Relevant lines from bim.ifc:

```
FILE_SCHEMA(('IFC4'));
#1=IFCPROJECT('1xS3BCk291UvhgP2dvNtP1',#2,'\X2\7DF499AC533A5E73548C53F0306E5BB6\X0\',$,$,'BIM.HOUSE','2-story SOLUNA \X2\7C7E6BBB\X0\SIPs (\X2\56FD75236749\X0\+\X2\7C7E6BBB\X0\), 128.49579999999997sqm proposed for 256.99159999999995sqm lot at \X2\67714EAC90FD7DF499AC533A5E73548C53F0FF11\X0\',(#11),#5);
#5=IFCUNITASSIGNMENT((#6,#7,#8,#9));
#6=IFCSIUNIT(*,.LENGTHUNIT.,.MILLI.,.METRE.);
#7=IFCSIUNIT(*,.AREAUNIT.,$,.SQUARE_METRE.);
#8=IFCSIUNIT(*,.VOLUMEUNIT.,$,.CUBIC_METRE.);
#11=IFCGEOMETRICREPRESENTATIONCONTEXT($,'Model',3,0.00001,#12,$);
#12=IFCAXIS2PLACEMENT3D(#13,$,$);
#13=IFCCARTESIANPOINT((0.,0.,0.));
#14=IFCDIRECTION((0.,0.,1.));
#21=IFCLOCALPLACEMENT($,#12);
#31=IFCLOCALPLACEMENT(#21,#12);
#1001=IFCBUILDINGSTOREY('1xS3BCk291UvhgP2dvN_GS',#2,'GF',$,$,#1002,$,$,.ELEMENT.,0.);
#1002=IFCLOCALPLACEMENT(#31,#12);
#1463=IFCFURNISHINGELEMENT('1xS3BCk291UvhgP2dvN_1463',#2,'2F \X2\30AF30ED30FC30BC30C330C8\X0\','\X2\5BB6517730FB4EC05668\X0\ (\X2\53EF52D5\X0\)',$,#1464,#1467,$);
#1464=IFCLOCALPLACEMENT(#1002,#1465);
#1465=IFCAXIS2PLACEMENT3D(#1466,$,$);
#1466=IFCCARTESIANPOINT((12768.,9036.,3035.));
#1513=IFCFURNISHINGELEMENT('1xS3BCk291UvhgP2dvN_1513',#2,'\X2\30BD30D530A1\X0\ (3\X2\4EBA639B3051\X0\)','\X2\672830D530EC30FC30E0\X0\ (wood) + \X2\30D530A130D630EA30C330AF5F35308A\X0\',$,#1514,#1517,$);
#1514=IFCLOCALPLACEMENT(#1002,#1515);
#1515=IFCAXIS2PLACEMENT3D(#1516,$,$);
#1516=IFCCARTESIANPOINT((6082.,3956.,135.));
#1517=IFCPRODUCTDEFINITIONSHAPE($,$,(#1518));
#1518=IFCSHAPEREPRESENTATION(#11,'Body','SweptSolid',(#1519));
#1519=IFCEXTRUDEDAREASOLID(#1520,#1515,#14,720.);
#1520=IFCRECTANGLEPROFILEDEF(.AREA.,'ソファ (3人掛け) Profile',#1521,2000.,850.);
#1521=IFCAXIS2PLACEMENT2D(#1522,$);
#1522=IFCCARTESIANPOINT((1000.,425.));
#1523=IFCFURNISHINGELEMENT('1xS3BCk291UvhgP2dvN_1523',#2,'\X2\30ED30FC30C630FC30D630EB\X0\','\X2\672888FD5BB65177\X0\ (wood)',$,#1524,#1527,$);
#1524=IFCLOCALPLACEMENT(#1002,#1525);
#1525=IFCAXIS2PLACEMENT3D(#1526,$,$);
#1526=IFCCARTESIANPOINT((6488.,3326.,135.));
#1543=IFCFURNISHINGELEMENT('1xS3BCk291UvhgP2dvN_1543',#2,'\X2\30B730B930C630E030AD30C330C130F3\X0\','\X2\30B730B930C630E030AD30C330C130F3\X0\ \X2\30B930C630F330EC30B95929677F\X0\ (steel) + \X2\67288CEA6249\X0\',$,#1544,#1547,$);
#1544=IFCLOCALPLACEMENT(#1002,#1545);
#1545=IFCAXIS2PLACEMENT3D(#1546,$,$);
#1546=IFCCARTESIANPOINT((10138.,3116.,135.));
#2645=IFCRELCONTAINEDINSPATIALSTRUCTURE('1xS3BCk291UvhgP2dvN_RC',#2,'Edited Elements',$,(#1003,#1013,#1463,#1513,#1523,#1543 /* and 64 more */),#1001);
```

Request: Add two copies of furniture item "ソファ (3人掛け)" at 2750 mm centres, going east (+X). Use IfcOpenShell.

```python
import numpy as np
import ifcopenshell
import ifcopenshell.api.geometry
import ifcopenshell.api.root
import ifcopenshell.util.element
import ifcopenshell.util.placement

model = ifcopenshell.open("bim.ifc")


def reuse_history(source, copy):
    """copy_class also copies each property set's owner history, people and application; keep the originals."""
    for rel in copy.IsDefinedBy:
        if rel.is_a("IfcRelDefinesByProperties") and (history := rel.RelatingPropertyDefinition.OwnerHistory):
            rel.RelatingPropertyDefinition.OwnerHistory = source.OwnerHistory
            ifcopenshell.util.element.remove_deep2(model, history)


source = model.by_id(1513)
base = ifcopenshell.util.placement.get_local_placement(source.ObjectPlacement)
step = np.array([1.0, 0.0, 0.0]) * 2750.0

for i in range(1, 3):
    copy = ifcopenshell.api.root.copy_class(model, product=source)
    copy.Representation = ifcopenshell.util.element.copy_deep(
        model, source.Representation, exclude=["IfcGeometricRepresentationContext", "IfcRepresentationMap"]
    )
    reuse_history(source, copy)
    matrix = base.copy()
    matrix[:3, 3] += i * step
    print("added at", matrix[:3, 3].round(3) + 0.0)
    ifcopenshell.api.geometry.edit_object_placement(model, product=copy, matrix=matrix, is_si=False)

model.write("bim-out.ifc")
```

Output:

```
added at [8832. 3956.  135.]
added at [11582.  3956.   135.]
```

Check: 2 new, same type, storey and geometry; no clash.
